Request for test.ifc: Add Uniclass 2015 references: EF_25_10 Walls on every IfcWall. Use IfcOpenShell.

First a look at what the model holds.

```python
import ifcopenshell

model = ifcopenshell.open("test.ifc")
print(model.schema)
print("classifications:", [c.Name for c in model.by_type("IfcClassification")])
for ifc_class in ("IfcDoor", "IfcRoof", "IfcStair", "IfcWall", "IfcWindow"):
    print(ifc_class, len(model.by_type(ifc_class)))
```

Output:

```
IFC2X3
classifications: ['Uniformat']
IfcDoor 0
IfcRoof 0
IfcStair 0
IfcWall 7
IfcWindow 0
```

```python
import ifcopenshell
import ifcopenshell.api.classification

model = ifcopenshell.open("test.ifc")

# IFC2X3 requires Source and Edition and has no link from the project to the system.
system = model.create_entity("IfcClassification", Source="NBS", Edition="2015", Name="Uniclass 2015")

codes = {
    "IfcWall": ("EF_25_10", "Walls"),
}
for ifc_class, (code, name) in codes.items():
    products = model.by_type(ifc_class)
    ifcopenshell.api.classification.add_reference(
        model, products=products, classification=system, identification=code, name=name
    )
    print(code, len(products))

model.write("test_updated.ifc")
```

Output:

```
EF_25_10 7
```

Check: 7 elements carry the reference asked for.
